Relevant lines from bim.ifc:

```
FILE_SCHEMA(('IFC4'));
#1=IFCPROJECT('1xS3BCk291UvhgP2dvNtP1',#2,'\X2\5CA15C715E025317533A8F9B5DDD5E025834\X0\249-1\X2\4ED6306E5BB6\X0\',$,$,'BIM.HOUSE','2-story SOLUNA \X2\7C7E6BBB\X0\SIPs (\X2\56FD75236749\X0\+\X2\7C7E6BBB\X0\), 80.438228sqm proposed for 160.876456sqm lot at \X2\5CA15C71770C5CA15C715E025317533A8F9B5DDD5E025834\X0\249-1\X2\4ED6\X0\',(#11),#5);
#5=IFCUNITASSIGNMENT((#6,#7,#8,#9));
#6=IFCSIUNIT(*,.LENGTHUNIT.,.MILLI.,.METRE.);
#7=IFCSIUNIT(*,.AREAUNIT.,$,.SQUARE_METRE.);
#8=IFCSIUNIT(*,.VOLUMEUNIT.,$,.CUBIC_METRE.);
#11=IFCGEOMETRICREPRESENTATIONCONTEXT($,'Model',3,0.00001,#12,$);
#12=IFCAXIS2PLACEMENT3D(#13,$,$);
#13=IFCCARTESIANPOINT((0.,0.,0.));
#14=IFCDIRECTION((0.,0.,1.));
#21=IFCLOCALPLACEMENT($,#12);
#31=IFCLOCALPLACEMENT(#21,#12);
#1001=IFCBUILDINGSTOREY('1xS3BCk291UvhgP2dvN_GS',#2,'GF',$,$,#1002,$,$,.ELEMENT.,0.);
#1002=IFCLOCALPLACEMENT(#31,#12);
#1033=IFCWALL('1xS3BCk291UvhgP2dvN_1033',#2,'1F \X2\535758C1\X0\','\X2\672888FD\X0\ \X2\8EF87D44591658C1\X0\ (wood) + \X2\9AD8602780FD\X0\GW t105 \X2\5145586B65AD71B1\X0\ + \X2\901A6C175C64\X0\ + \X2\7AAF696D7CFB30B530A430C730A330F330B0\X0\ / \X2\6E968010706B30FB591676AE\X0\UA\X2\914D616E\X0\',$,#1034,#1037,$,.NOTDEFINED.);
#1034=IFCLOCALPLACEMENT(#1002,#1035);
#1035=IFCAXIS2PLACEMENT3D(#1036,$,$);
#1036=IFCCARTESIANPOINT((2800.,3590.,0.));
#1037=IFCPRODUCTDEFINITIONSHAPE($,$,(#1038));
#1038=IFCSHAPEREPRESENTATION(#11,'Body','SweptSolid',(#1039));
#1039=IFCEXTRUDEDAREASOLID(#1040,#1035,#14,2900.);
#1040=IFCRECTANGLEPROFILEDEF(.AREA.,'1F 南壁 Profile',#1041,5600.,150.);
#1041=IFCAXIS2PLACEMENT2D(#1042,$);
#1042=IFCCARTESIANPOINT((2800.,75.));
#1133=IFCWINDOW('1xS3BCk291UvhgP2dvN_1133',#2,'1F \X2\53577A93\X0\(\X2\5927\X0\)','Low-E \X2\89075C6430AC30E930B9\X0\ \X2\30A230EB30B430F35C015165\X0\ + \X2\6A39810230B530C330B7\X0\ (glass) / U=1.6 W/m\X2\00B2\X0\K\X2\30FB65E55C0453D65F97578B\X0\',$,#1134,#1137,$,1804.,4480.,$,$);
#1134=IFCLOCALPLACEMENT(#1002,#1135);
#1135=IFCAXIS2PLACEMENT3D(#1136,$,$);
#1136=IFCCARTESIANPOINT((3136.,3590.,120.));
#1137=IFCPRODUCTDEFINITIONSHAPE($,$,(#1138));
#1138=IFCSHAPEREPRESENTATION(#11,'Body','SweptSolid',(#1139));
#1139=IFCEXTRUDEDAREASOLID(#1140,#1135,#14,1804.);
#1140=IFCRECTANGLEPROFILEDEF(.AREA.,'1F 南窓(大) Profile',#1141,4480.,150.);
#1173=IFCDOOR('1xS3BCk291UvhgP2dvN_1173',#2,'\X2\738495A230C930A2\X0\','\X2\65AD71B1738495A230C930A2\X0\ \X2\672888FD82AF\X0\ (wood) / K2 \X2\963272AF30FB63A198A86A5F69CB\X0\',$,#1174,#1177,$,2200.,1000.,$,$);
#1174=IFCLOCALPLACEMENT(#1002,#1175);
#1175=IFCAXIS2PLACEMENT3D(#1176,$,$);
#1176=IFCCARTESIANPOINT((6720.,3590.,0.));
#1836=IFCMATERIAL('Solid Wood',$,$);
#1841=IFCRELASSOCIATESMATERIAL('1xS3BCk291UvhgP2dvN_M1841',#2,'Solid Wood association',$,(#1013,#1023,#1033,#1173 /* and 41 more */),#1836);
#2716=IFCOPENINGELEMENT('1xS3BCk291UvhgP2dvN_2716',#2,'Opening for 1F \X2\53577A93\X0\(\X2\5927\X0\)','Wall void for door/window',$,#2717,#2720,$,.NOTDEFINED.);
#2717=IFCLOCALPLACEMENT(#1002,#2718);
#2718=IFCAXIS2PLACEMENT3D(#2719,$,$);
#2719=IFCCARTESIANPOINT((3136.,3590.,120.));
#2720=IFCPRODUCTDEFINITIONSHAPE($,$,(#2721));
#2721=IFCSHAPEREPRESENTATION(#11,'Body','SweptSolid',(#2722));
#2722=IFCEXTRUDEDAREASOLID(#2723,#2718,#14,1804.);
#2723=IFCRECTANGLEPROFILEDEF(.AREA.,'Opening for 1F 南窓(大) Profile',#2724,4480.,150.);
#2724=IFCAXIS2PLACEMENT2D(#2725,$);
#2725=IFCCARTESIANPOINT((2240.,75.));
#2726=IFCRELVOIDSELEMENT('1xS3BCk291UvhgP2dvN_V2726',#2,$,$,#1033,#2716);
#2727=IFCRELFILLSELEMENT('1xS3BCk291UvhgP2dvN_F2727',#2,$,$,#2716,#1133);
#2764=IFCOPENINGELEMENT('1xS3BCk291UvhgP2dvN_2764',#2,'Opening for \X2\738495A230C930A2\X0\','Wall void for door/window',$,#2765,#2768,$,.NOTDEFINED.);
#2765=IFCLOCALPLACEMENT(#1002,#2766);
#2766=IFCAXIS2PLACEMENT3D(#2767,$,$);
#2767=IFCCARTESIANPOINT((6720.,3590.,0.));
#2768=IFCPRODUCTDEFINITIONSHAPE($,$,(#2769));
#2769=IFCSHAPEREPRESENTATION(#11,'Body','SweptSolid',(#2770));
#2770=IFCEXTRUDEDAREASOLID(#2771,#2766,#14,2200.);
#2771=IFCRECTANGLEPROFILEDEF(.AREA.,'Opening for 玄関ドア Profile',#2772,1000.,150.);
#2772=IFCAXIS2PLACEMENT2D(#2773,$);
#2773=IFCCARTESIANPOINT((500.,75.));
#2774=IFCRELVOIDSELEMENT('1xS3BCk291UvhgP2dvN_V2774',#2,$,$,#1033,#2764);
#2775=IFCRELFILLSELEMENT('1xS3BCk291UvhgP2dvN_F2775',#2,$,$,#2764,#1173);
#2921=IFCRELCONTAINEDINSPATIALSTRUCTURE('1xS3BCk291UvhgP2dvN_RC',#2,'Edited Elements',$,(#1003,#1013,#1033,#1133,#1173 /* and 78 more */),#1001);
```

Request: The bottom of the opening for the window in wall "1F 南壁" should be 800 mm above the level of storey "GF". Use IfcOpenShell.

```python
import numpy as np
import ifcopenshell
import ifcopenshell.api.geometry
import ifcopenshell.geom
import ifcopenshell.util.element
import ifcopenshell.util.placement
import ifcopenshell.util.shape
import ifcopenshell.util.unit

model = ifcopenshell.open("bim.ifc")
unit_scale = ifcopenshell.util.unit.calculate_unit_scale(model)

window = model.by_guid("1xS3BCk291UvhgP2dvN_1133")
opening = window.FillsVoids[0].RelatingOpeningElement
storey = ifcopenshell.util.element.get_container(window, ifc_class="IfcBuildingStorey")
level = ifcopenshell.util.placement.get_local_placement(storey.ObjectPlacement)[2, 3]

# The opening's origin need not be at the sill, so measure its lowest point.
shape = ifcopenshell.geom.create_shape(ifcopenshell.geom.settings(), opening)
bottom = ifcopenshell.util.shape.get_shape_bottom_elevation(shape, shape.geometry) / unit_scale
dz = level + 800.0 - bottom

shift = np.array([0.0, 0.0, dz])
# The window is not placed relative to its opening, so move both.
for product in (opening, window):
    matrix = ifcopenshell.util.placement.get_local_placement(product.ObjectPlacement)
    matrix[:3, 3] += shift
    ifcopenshell.api.geometry.edit_object_placement(model, product=product, matrix=matrix, is_si=False)

print(f"moved by {dz * unit_scale:+.3f} m")

model.write("bim_v2.ifc")
```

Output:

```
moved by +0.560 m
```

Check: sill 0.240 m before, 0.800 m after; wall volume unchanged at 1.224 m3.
